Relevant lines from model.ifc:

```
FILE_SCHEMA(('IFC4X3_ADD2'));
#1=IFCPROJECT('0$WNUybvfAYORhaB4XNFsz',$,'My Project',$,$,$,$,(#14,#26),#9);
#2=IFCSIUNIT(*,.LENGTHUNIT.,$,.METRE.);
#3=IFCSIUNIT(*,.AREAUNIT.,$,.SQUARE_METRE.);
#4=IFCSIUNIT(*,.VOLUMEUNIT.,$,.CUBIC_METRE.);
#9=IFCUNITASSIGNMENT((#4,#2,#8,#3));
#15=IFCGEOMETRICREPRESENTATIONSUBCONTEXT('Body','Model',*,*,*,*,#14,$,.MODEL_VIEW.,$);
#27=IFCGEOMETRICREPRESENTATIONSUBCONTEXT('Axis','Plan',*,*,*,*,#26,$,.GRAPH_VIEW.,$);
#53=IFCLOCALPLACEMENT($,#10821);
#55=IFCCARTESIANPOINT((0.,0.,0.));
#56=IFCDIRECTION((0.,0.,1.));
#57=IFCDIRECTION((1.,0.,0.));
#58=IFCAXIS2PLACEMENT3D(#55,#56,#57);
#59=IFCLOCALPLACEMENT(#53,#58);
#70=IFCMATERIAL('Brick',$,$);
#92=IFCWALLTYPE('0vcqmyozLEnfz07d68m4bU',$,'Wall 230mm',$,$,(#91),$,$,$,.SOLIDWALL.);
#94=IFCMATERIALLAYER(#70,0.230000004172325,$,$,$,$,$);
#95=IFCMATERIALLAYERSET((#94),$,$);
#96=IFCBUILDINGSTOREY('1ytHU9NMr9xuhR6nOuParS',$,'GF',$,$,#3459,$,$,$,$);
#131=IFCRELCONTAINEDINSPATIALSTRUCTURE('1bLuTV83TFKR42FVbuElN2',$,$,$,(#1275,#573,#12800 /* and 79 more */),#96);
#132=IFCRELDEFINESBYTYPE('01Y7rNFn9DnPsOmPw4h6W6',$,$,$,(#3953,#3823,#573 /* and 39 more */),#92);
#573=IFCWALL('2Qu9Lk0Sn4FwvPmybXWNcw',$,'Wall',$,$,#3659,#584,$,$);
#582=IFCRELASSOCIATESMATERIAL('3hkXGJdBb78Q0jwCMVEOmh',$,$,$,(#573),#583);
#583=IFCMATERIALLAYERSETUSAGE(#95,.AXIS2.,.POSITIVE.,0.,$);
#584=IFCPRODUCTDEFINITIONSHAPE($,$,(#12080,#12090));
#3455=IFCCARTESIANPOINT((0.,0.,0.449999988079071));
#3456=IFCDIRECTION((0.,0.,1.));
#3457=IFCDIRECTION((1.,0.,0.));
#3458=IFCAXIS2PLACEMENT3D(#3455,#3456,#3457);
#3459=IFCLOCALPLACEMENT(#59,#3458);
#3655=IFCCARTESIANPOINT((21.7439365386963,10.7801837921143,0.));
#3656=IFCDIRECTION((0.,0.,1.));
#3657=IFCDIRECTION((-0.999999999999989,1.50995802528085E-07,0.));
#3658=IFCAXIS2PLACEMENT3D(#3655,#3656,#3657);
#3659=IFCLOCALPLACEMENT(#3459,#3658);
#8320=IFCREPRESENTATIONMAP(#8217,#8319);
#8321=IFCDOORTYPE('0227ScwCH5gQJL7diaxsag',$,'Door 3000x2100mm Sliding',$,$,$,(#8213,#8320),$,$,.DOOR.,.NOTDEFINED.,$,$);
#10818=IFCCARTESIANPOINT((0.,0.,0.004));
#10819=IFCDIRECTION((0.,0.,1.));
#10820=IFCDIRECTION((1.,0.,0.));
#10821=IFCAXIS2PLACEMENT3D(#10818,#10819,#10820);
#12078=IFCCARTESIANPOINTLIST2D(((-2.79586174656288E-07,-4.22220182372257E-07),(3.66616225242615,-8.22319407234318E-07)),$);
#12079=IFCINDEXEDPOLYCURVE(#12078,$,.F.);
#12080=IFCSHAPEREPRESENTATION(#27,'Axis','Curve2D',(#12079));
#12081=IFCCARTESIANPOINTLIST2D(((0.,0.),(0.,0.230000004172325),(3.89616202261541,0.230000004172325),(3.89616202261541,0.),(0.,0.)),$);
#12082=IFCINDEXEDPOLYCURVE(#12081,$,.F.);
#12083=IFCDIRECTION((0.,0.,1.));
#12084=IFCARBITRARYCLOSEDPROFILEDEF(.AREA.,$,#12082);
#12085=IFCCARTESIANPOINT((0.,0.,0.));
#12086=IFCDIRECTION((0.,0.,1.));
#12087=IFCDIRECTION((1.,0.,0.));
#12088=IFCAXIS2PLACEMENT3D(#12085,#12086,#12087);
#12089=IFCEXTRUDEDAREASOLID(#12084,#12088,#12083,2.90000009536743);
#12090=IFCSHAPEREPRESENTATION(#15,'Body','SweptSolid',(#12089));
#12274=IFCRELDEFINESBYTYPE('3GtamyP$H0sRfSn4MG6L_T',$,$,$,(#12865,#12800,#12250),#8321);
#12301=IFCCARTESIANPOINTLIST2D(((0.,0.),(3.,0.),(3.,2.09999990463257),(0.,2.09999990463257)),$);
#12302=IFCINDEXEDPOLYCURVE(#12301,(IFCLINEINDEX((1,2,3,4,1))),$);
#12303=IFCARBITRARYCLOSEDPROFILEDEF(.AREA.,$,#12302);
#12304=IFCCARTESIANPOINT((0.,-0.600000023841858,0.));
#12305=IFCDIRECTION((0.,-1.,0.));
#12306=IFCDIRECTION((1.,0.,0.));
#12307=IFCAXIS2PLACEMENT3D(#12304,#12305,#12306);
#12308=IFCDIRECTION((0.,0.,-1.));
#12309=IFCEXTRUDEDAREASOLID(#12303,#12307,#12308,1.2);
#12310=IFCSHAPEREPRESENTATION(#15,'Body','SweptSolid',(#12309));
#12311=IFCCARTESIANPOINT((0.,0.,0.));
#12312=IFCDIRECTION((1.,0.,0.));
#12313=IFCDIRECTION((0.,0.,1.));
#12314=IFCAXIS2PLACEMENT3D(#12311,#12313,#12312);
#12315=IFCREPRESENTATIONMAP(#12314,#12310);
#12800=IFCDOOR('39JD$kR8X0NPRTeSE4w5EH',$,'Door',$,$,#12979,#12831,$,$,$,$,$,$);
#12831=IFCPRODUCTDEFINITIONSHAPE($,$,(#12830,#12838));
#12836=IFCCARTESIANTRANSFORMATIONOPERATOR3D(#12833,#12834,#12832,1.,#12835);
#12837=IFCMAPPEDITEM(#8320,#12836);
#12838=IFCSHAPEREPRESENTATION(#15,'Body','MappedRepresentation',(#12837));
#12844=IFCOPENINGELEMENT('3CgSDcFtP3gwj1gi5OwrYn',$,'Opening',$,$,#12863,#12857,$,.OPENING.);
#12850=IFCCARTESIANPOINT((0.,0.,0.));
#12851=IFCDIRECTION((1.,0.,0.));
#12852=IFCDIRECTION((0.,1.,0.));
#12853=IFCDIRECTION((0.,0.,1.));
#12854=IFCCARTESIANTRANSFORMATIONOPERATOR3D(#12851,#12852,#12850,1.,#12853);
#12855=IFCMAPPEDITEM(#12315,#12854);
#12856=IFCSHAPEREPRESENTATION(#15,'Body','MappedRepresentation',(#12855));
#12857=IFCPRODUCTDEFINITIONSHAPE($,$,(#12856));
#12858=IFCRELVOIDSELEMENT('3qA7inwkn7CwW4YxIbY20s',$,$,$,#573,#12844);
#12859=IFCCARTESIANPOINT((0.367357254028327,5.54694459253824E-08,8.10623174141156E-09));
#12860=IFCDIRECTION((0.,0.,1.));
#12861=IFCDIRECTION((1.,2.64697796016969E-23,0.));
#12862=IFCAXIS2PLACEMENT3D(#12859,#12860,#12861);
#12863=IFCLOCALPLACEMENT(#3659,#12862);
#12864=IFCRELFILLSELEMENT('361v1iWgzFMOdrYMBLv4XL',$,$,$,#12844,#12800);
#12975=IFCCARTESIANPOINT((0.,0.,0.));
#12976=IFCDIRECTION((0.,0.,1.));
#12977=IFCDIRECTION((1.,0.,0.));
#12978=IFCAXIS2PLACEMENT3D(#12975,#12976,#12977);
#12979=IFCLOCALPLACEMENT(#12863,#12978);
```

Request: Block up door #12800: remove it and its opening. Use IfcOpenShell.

```python
import ifcopenshell
import ifcopenshell.api.feature
import ifcopenshell.api.root
import ifcopenshell.geom
import ifcopenshell.util.shape

model = ifcopenshell.open("model.ifc")
settings = ifcopenshell.geom.settings()


def volume(element):
    """Net volume in cubic metres, openings subtracted."""
    shape = ifcopenshell.geom.create_shape(settings, element)
    return ifcopenshell.util.shape.get_volume(shape.geometry)


door = model.by_id(12800)
opening = door.FillsVoids[0].RelatingOpeningElement
wall = opening.VoidsElements[0].RelatingBuildingElement
before = volume(wall)

ifcopenshell.api.root.remove_product(model, product=door)
ifcopenshell.api.feature.remove_feature(model, feature=opening)

after = volume(wall)

print(f"wall volume {before:.3f} -> {after:.3f} m3")

model.write("model_rev.ifc")
```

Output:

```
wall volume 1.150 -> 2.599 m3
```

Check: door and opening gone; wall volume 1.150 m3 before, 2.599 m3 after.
